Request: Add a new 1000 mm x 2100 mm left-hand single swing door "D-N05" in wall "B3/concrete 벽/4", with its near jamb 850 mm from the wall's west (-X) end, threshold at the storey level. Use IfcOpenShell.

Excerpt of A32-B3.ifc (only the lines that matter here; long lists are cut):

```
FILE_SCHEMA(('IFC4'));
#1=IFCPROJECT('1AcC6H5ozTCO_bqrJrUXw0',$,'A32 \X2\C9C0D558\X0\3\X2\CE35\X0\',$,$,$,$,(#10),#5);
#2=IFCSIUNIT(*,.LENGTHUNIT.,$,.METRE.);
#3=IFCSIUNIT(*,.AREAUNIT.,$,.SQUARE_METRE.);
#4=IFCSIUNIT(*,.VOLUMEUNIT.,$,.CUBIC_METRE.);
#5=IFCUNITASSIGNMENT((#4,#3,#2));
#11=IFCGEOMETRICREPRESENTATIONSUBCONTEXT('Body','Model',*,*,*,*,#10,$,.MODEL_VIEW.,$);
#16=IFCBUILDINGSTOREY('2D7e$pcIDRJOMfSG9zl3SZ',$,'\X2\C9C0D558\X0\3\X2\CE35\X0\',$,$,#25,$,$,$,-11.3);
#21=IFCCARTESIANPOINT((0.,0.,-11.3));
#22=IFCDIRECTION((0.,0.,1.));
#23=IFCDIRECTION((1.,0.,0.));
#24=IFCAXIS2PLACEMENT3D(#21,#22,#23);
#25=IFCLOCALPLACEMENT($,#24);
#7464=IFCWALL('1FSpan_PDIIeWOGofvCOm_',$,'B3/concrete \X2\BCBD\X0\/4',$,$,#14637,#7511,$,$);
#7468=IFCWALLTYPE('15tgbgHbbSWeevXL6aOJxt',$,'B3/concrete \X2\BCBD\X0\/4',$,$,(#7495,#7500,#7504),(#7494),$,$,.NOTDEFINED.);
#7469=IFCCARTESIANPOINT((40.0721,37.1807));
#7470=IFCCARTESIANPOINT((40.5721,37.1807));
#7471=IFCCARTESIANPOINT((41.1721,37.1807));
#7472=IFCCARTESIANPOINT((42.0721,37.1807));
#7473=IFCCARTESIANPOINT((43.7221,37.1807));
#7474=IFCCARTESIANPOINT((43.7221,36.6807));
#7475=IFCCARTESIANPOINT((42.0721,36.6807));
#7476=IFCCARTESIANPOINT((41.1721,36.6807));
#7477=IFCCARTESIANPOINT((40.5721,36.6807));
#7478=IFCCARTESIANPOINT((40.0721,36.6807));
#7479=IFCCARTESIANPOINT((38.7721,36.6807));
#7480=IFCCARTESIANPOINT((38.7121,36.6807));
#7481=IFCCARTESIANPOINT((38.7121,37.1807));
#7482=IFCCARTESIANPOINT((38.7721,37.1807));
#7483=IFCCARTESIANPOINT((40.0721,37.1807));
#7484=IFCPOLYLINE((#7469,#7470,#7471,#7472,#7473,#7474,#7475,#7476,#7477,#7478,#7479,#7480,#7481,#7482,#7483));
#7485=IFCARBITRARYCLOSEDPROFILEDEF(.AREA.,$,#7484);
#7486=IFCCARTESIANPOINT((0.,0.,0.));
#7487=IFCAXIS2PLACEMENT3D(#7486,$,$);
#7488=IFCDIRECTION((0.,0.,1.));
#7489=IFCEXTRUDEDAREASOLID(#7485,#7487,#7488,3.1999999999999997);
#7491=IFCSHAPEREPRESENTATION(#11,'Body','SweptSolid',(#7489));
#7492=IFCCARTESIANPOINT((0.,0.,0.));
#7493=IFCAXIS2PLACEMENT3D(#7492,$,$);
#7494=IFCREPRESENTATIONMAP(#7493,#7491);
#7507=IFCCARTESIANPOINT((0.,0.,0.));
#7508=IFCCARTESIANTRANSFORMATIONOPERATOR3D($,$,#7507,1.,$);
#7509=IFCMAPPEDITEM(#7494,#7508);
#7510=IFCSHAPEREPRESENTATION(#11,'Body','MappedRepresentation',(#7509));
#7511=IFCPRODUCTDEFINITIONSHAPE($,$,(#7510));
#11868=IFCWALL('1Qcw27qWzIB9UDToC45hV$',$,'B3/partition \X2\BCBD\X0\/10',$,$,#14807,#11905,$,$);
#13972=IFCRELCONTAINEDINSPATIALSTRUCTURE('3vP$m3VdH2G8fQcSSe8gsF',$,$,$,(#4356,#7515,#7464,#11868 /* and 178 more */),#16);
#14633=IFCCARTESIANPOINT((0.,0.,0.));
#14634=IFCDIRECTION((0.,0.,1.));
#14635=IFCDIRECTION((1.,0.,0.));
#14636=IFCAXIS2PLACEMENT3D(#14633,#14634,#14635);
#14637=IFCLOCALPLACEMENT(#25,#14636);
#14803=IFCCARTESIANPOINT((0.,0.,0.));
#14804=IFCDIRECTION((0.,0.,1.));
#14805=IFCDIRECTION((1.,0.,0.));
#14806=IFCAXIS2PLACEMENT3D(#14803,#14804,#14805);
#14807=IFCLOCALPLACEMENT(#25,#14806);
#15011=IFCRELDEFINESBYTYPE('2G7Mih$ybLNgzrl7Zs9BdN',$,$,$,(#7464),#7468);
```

```python
import numpy as np
import ifcopenshell
import ifcopenshell.api.feature
import ifcopenshell.api.geometry
import ifcopenshell.api.root
import ifcopenshell.api.spatial
import ifcopenshell.geom
import ifcopenshell.util.element
import ifcopenshell.util.placement
import ifcopenshell.util.representation
import ifcopenshell.util.shape
import ifcopenshell.util.unit

model = ifcopenshell.open("A32-B3.ifc")
unit_scale = ifcopenshell.util.unit.calculate_unit_scale(model)
settings = ifcopenshell.geom.settings()


def volume(element):
    """Net volume in cubic metres, openings subtracted."""
    shape = ifcopenshell.geom.create_shape(settings, element)
    return ifcopenshell.util.shape.get_volume(shape.geometry)


wall = model.by_guid("1FSpan_PDIIeWOGofvCOm_")
storey = ifcopenshell.util.element.get_container(wall, ifc_class="IfcBuildingStorey")
context = ifcopenshell.util.representation.get_context(model, "Model", "Body", "MODEL_VIEW")
before = volume(wall)

width, height, from_end, sill = 1, 2.1, 0.85, 0.0  # metres

# The wall runs along its own X axis, and the end named is its -X end.
wall_shape = ifcopenshell.geom.create_shape(settings, wall)
x, y, z = ifcopenshell.util.shape.get_vertices(wall_shape.geometry).T
start = x.min() + from_end
face, thickness = float(y.min()), float(y.max() - y.min())
wall_matrix = ifcopenshell.util.placement.get_local_placement(wall.ObjectPlacement)
level = ifcopenshell.util.placement.get_local_placement(storey.ObjectPlacement)[2, 3]


def in_wall(x, y):
    """Placement at x, y metres in the wall's axes, at sill height."""
    matrix = wall_matrix.copy()
    matrix[:, 3] = wall_matrix @ np.array([x / unit_scale, y / unit_scale, 0.0, 1.0])
    matrix[2, 3] = level + sill / unit_scale
    return matrix


# Opening: a box that overshoots both wall faces by 50 mm.
opening = ifcopenshell.api.root.create_entity(model, ifc_class="IfcOpeningElement", predefined_type="OPENING")
box = ifcopenshell.api.geometry.add_wall_representation(
    model, context=context, length=width, height=height, thickness=thickness + 0.1
)
ifcopenshell.api.geometry.assign_representation(model, product=opening, representation=box)
ifcopenshell.api.geometry.edit_object_placement(model, product=opening, matrix=in_wall(start, face - 0.05), is_si=False)
ifcopenshell.api.feature.add_feature(model, feature=opening, element=wall)

door = ifcopenshell.api.root.create_entity(model, ifc_class="IfcDoor", name="D-N05", predefined_type="DOOR")
door.OverallWidth, door.OverallHeight = width / unit_scale, height / unit_scale
door.OperationType = "SINGLE_SWING_LEFT"
body = ifcopenshell.api.geometry.add_door_representation(
    model,
    context=context,
    overall_width=door.OverallWidth,
    overall_height=door.OverallHeight,
    operation_type="SINGLE_SWING_LEFT",
    lining_properties={"LiningDepth": thickness / unit_scale, "ThresholdDepth": thickness / unit_scale},
)
ifcopenshell.api.geometry.assign_representation(model, product=door, representation=body)
ifcopenshell.api.spatial.assign_container(model, products=[door], relating_structure=storey)
ifcopenshell.api.feature.add_filling(model, opening=opening, element=door)

# The lining spans the wall, so the door starts at the wall face.
ifcopenshell.api.geometry.edit_object_placement(model, product=door, matrix=in_wall(start, face), is_si=False)

after = volume(wall)

print(f"wall volume {before:.3f} -> {after:.3f} m3")

model.write("A32-B3_edited.ifc")
```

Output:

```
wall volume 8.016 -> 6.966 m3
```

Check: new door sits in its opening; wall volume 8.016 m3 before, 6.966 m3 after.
